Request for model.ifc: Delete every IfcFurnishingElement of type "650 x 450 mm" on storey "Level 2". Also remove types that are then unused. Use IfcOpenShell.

First a look at what the model holds.

```python
import ifcopenshell
import ifcopenshell.util.element

model = ifcopenshell.open("model.ifc")
print(model.schema)
storey = next(s for s in model.by_type("IfcBuildingStorey") if s.Name == "Level 2")
furniture = [e for e in ifcopenshell.util.element.get_decomposition(storey) if e.is_a("IfcFurnishingElement")]
seen = {}
for e in furniture:
    element_type = ifcopenshell.util.element.get_type(e)
    name = element_type.Name if element_type not in (None, e) else None
    seen[name] = seen.get(name, 0) + 1
for name, count in sorted(seen.items(), key=str):
    print(count, "x", name)
```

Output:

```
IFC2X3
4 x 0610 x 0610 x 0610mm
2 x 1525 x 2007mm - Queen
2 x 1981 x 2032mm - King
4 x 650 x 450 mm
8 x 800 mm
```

```python
import ifcopenshell
import ifcopenshell.api.root
import ifcopenshell.util.element

model = ifcopenshell.open("model.ifc")

storey = next(s for s in model.by_type("IfcBuildingStorey") if s.Name == "Level 2")
furniture = [e for e in ifcopenshell.util.element.get_decomposition(storey) if e.is_a("IfcFurnishingElement")]
targets = [e for e in furniture if (t := ifcopenshell.util.element.get_type(e)) not in (None, e) and t.Name == "650 x 450 mm"]
types = {ifcopenshell.util.element.get_type(e) for e in targets} - {None, *targets}

for e in targets:
    ifcopenshell.api.root.remove_product(model, product=e)
print(len(targets), "removed")

unused = [t for t in types if not ifcopenshell.util.element.get_types(t)]
for t in unused:
    ifcopenshell.api.root.remove_product(model, product=t)
print(len(unused), "unused types removed")

model.write("model_updated.ifc")
```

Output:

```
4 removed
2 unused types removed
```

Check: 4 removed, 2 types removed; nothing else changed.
